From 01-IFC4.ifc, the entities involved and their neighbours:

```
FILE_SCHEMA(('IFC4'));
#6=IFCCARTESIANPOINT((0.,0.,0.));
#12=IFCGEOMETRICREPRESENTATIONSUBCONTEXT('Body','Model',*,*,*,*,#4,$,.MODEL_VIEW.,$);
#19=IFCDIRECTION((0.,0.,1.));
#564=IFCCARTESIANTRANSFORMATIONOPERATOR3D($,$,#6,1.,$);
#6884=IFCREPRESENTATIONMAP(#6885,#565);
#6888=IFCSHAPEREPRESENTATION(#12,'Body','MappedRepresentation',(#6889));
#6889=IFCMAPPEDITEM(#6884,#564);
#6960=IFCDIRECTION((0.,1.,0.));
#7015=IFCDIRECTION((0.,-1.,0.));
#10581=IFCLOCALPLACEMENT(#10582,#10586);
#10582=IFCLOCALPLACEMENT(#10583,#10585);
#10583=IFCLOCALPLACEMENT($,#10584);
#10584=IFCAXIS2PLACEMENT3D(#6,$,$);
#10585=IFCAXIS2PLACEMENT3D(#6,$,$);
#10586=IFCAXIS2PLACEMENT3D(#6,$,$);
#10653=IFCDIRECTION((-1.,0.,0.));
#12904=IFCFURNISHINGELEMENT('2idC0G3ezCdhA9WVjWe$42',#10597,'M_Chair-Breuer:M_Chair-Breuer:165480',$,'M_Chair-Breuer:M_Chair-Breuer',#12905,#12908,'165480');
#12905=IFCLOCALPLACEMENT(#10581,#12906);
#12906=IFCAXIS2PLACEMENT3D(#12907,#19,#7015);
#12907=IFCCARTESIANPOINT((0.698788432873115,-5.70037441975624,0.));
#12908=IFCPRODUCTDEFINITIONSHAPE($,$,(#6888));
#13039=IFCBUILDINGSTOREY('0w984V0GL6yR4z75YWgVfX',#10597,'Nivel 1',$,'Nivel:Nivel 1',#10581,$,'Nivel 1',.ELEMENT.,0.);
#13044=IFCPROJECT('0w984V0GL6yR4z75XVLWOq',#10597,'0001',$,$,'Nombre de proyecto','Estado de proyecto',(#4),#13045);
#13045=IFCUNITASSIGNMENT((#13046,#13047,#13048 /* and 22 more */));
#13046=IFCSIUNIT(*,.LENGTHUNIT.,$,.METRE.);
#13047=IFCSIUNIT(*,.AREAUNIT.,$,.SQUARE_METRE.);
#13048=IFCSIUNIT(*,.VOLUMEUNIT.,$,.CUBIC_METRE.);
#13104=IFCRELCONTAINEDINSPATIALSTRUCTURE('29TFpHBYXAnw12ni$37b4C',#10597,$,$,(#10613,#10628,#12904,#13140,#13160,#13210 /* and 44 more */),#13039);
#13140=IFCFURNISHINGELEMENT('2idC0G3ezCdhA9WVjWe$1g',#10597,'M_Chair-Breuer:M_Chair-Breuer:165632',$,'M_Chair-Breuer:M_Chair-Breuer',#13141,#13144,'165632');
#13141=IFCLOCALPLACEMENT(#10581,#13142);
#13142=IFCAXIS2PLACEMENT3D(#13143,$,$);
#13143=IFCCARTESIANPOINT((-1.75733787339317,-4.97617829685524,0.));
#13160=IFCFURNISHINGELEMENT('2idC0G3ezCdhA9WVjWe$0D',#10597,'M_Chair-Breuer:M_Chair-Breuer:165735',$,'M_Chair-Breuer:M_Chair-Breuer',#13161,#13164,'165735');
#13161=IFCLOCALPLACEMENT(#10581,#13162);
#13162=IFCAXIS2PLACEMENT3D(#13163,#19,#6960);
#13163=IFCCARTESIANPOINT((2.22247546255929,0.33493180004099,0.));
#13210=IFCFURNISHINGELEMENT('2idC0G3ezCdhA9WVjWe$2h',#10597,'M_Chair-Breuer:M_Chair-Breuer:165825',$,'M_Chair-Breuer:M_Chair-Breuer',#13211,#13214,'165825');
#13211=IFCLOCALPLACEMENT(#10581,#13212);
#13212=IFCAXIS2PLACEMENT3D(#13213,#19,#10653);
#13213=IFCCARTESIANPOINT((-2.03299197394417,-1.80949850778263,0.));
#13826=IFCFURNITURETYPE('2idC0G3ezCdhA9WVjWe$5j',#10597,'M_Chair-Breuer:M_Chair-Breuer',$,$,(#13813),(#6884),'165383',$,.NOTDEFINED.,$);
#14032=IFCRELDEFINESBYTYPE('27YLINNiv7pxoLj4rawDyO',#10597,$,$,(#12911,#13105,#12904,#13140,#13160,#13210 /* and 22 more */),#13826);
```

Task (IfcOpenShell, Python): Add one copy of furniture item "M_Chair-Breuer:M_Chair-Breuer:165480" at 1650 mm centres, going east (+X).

```python
import numpy as np
import ifcopenshell
import ifcopenshell.api.geometry
import ifcopenshell.api.root
import ifcopenshell.util.element
import ifcopenshell.util.placement

model = ifcopenshell.open("01-IFC4.ifc")


def reuse_history(source, copy):
    """copy_class also copies each property set's owner history, people and application; keep the originals."""
    for rel in copy.IsDefinedBy:
        if rel.is_a("IfcRelDefinesByProperties") and (history := rel.RelatingPropertyDefinition.OwnerHistory):
            rel.RelatingPropertyDefinition.OwnerHistory = source.OwnerHistory
            ifcopenshell.util.element.remove_deep2(model, history)


source = model.by_guid("2idC0G3ezCdhA9WVjWe$42")
base = ifcopenshell.util.placement.get_local_placement(source.ObjectPlacement)
step = np.array([1.0, 0.0, 0.0]) * 1.65

for i in range(1, 2):
    copy = ifcopenshell.api.root.copy_class(model, product=source)
    copy.Representation = ifcopenshell.util.element.copy_deep(
        model, source.Representation, exclude=["IfcGeometricRepresentationContext", "IfcRepresentationMap"]
    )
    copy.Name = "M_Chair-Breuer:M_Chair-Breuer"
    copy.Tag = None
    reuse_history(source, copy)
    matrix = base.copy()
    matrix[:3, 3] += i * step
    print("added at", matrix[:3, 3].round(3) + 0.0)
    ifcopenshell.api.geometry.edit_object_placement(model, product=copy, matrix=matrix, is_si=False)

model.write("01-IFC4_rev.ifc")
```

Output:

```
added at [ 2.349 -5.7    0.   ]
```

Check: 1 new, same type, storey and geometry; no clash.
